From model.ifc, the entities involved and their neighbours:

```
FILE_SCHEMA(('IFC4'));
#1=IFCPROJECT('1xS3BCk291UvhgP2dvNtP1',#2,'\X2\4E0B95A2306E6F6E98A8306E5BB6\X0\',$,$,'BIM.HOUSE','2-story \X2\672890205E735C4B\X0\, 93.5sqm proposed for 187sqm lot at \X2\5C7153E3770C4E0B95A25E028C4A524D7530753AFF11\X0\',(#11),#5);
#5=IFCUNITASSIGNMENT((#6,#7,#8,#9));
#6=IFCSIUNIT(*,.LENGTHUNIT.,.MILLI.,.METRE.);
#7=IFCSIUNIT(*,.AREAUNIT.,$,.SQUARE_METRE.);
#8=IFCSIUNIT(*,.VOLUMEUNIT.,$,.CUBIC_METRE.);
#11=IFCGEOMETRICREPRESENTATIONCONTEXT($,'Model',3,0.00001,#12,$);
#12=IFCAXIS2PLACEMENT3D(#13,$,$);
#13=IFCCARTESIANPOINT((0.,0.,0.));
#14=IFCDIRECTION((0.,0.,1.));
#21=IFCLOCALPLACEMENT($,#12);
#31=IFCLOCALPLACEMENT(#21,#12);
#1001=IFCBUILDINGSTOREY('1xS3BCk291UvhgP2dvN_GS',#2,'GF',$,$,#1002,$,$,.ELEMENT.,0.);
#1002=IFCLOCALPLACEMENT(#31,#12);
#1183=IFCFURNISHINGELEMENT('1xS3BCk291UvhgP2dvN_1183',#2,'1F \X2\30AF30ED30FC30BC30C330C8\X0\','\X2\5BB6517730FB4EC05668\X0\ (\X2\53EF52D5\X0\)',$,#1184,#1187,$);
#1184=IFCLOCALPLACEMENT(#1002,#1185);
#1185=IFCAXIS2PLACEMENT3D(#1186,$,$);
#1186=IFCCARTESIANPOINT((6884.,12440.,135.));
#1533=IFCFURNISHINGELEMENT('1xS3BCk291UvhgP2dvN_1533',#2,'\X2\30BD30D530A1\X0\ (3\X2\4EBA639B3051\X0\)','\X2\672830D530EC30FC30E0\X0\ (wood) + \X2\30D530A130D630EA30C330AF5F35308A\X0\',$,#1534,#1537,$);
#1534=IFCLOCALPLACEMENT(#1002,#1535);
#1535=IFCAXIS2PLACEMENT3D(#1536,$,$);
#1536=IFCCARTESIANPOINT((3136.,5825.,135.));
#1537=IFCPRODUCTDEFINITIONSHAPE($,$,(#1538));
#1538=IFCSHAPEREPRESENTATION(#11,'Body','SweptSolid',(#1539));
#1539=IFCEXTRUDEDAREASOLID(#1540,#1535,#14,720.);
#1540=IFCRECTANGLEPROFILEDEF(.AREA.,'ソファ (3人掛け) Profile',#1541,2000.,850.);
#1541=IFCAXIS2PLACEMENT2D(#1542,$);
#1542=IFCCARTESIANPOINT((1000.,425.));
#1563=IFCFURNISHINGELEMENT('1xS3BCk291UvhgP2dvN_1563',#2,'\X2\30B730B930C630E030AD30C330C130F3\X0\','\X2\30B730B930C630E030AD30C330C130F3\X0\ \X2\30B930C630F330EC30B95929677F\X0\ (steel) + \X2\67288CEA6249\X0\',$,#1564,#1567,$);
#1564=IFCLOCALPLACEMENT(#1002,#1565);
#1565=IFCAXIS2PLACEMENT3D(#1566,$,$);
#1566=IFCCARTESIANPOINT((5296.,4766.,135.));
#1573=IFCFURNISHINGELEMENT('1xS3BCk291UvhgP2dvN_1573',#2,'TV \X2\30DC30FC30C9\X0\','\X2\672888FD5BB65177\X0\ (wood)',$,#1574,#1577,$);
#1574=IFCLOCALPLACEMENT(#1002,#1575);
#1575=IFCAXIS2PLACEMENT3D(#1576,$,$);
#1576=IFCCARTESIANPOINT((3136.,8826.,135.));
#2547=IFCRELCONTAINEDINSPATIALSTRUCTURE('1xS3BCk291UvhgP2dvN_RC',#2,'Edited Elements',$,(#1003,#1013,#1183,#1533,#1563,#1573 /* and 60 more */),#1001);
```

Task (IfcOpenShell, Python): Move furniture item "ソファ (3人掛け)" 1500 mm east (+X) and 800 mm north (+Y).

```python
import ifcopenshell
import ifcopenshell.api.geometry
import ifcopenshell.util.placement

model = ifcopenshell.open("model.ifc")

item = model.by_guid("1xS3BCk291UvhgP2dvN_1533")
matrix = ifcopenshell.util.placement.get_local_placement(item.ObjectPlacement)
matrix[0, 3] += 1500.0
matrix[1, 3] += 800.0
ifcopenshell.api.geometry.edit_object_placement(model, product=item, matrix=matrix, is_si=False)

print(ifcopenshell.util.placement.get_local_placement(item.ObjectPlacement).round(3) + 0.0)

model.write("model_v2.ifc")
```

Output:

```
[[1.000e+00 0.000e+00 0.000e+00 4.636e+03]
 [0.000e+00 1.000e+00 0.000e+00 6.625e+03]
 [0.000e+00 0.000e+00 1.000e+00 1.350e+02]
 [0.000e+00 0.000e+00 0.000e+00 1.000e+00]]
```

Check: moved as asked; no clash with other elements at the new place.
